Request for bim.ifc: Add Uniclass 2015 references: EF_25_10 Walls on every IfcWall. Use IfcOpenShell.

First a look at what the model holds.

```python
import ifcopenshell

model = ifcopenshell.open("bim.ifc")
print(model.schema)
print("classifications:", [c.Name for c in model.by_type("IfcClassification")])
for ifc_class in ("IfcDoor", "IfcRoof", "IfcStair", "IfcWall", "IfcWindow"):
    print(ifc_class, len(model.by_type(ifc_class)))
```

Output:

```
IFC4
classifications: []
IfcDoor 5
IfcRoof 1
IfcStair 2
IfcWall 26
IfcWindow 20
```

```python
import ifcopenshell
import ifcopenshell.api.classification

model = ifcopenshell.open("bim.ifc")

system = ifcopenshell.api.classification.add_classification(model, classification="Uniclass 2015")

codes = {
    "IfcWall": ("EF_25_10", "Walls"),
}
for ifc_class, (code, name) in codes.items():
    products = model.by_type(ifc_class)
    ifcopenshell.api.classification.add_reference(
        model, products=products, classification=system, identification=code, name=name
    )
    print(code, len(products))

model.write("bim-out.ifc")
```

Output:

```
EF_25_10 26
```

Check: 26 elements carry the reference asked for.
